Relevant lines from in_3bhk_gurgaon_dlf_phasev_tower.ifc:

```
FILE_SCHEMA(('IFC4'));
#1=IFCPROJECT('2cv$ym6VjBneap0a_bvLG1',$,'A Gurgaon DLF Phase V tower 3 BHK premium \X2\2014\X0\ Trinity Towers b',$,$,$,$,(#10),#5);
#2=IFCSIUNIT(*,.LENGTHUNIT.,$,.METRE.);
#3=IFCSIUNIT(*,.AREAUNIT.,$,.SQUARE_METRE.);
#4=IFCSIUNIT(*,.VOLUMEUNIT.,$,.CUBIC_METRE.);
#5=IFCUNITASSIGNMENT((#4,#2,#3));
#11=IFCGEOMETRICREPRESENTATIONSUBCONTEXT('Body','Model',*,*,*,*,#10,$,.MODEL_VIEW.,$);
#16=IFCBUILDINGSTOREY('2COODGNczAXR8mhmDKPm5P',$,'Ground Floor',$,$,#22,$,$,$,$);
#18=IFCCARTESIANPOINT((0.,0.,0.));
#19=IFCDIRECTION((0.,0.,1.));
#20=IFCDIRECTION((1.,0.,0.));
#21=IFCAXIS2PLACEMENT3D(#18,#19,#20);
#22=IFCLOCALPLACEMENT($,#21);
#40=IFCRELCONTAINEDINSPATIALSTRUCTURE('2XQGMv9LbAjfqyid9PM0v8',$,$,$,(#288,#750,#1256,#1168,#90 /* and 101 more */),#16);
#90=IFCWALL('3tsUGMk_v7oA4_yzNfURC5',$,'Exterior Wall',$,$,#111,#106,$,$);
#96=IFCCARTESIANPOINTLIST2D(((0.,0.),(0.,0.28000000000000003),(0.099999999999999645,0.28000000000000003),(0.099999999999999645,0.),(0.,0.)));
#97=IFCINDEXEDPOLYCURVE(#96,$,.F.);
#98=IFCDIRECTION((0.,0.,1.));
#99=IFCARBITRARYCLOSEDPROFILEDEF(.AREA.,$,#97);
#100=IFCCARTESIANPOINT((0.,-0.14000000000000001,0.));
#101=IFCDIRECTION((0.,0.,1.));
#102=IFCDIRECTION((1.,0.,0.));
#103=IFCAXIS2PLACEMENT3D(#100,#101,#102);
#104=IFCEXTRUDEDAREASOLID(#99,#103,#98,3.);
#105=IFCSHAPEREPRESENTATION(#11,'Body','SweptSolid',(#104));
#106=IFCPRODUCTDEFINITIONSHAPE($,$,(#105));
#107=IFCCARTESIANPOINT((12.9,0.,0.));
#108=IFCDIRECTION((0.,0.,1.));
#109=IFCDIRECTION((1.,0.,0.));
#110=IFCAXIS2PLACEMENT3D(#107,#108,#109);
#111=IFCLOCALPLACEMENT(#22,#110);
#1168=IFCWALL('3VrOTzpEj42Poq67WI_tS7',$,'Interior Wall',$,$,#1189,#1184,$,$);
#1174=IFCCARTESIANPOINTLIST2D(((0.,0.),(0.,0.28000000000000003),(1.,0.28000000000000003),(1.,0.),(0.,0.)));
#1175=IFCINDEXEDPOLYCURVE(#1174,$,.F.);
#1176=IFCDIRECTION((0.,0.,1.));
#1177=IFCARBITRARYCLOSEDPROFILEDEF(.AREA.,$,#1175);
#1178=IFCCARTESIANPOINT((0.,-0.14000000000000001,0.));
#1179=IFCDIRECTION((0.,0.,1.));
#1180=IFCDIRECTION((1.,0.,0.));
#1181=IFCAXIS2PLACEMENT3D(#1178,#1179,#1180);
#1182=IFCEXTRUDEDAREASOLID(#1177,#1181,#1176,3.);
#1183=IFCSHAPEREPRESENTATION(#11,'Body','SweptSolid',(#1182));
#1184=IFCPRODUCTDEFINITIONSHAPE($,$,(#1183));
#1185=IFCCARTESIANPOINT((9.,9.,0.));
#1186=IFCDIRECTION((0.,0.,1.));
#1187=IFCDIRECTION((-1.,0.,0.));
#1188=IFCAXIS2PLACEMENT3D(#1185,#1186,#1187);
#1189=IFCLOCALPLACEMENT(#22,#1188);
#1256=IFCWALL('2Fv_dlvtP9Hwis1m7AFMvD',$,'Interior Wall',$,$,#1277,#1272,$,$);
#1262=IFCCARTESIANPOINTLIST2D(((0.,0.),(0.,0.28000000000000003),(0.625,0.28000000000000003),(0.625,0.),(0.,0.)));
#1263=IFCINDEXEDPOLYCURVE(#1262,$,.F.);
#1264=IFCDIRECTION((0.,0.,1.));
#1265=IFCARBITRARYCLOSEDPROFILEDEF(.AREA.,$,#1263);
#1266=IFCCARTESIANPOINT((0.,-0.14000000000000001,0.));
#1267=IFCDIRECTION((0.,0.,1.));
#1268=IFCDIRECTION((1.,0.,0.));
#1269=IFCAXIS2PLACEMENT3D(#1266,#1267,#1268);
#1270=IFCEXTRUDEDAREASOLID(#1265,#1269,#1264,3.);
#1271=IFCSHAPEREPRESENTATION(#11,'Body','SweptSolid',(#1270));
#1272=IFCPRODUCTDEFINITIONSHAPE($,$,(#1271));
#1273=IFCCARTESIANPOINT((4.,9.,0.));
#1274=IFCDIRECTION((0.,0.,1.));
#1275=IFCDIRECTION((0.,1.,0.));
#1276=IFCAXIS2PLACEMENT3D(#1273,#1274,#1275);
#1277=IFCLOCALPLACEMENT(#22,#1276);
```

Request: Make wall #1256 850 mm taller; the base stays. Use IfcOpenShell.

```python
import ifcopenshell
import ifcopenshell.geom
import ifcopenshell.util.representation
import ifcopenshell.util.shape
import ifcopenshell.util.unit

model = ifcopenshell.open("in_3bhk_gurgaon_dlf_phasev_tower.ifc")
unit_scale = ifcopenshell.util.unit.calculate_unit_scale(model)
settings = ifcopenshell.geom.settings()


def volume(element):
    """Net volume in cubic metres, openings subtracted."""
    shape = ifcopenshell.geom.create_shape(settings, element)
    return ifcopenshell.util.shape.get_volume(shape.geometry)


wall = model.by_guid("2Fv_dlvtP9Hwis1m7AFMvD")
before = volume(wall)

body = ifcopenshell.util.representation.get_representation(wall, "Model", "Body")
solid = body.Items[0]
old_height = solid.Depth
solid.Depth += 0.85 / unit_scale
after = volume(wall)

print(f"height {old_height:g} -> {solid.Depth:g}, volume {before:.3f} -> {after:.3f} m3")

model.write("in_3bhk_gurgaon_dlf_phasev_tower_updated.ifc")
```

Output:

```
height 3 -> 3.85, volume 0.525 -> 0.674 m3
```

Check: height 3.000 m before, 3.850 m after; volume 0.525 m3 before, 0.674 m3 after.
